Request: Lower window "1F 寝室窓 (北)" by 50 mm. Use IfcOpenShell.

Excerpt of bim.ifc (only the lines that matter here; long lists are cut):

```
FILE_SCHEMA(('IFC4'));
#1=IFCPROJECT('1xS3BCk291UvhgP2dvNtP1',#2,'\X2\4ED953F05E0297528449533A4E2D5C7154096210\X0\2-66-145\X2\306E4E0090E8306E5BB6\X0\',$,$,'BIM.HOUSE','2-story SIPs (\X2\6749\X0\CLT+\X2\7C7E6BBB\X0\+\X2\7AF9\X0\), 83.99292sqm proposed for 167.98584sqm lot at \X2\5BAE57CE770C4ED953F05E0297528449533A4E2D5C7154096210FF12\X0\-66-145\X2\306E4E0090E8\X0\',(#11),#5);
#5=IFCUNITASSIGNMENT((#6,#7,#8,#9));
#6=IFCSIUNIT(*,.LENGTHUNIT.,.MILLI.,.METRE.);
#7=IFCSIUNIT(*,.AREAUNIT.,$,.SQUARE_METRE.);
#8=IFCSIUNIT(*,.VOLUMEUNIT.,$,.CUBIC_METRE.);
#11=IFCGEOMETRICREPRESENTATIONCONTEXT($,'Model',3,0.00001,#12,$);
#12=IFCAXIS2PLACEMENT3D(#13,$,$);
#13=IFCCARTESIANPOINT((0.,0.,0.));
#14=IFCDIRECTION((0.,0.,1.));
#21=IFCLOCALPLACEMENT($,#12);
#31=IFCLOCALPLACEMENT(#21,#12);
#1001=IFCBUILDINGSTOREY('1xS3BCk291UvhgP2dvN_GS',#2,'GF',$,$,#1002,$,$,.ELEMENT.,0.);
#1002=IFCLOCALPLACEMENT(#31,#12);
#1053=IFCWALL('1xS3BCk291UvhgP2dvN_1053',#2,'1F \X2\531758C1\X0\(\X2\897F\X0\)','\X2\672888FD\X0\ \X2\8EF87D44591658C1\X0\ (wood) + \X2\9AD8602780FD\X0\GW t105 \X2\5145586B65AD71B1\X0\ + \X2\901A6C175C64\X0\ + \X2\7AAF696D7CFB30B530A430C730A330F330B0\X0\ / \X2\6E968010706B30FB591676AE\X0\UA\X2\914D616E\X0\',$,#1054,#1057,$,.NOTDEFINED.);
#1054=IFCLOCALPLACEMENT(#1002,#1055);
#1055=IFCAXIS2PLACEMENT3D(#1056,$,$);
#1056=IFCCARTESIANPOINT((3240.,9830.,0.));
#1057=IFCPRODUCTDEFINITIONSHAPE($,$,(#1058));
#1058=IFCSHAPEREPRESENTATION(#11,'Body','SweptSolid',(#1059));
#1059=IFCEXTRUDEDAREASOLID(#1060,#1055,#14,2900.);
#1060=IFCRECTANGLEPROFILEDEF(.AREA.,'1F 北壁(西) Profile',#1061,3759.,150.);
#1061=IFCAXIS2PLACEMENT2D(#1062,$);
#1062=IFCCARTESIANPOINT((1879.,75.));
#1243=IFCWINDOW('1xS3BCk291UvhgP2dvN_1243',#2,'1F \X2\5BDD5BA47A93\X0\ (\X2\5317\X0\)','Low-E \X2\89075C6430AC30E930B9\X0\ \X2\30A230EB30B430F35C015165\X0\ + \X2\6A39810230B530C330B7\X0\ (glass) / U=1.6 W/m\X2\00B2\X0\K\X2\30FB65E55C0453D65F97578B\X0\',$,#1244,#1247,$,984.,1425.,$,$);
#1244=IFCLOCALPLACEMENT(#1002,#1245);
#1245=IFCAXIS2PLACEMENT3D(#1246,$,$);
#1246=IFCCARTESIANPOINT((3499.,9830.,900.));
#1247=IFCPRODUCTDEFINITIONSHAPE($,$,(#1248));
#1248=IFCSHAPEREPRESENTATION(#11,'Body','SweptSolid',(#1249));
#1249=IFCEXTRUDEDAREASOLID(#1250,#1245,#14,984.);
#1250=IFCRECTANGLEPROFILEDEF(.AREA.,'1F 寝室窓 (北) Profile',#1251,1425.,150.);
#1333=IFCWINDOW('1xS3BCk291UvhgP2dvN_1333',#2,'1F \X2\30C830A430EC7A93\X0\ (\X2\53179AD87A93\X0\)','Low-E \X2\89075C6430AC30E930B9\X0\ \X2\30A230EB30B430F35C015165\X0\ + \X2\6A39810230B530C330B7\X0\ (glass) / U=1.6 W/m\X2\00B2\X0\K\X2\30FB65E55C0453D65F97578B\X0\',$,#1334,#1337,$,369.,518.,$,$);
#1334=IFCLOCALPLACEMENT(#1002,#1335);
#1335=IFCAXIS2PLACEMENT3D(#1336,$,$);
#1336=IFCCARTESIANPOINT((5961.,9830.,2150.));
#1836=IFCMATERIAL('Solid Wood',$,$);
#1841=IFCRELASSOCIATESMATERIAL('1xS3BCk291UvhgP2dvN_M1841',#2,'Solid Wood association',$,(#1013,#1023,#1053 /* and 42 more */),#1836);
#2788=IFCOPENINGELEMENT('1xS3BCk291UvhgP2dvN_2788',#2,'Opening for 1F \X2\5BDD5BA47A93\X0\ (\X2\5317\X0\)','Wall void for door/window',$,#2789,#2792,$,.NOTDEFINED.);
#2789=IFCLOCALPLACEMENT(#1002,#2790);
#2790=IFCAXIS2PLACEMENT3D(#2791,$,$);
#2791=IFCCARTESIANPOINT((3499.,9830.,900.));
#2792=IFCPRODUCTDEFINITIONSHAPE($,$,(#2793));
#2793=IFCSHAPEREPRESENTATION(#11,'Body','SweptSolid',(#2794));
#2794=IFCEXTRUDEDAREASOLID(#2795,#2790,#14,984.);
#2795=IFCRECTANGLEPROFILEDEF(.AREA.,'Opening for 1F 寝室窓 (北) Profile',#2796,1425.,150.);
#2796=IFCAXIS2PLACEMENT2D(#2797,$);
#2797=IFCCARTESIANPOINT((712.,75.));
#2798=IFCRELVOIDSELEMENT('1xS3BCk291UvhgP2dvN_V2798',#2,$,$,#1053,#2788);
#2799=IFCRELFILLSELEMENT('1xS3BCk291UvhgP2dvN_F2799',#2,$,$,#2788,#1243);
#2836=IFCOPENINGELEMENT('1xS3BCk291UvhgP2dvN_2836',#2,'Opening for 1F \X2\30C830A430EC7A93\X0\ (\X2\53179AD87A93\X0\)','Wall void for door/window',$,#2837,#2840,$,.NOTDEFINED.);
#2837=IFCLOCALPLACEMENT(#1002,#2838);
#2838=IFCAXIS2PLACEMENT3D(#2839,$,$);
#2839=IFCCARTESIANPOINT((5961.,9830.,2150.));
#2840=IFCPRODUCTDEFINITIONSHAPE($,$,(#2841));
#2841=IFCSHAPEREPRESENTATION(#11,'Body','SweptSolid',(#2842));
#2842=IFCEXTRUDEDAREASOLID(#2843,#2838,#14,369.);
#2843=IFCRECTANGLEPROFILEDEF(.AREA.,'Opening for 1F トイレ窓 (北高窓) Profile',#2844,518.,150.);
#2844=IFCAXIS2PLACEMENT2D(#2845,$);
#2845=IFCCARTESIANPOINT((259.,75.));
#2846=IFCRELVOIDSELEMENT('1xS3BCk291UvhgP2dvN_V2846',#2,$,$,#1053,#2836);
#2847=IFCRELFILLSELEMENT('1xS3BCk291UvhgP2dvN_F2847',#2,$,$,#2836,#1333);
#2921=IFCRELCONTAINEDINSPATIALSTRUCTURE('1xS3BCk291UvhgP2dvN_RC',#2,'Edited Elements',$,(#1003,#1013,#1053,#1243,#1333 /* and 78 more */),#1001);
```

```python
import numpy as np
import ifcopenshell
import ifcopenshell.api.geometry
import ifcopenshell.util.placement
import ifcopenshell.util.unit

model = ifcopenshell.open("bim.ifc")
unit_scale = ifcopenshell.util.unit.calculate_unit_scale(model)

window = model.by_guid("1xS3BCk291UvhgP2dvN_1243")
opening = window.FillsVoids[0].RelatingOpeningElement
dz = -50.0

shift = np.array([0.0, 0.0, dz])
# The window is not placed relative to its opening, so move both.
for product in (opening, window):
    matrix = ifcopenshell.util.placement.get_local_placement(product.ObjectPlacement)
    matrix[:3, 3] += shift
    ifcopenshell.api.geometry.edit_object_placement(model, product=product, matrix=matrix, is_si=False)

print(f"moved by {dz * unit_scale:+.3f} m")

model.write("bim_edited.ifc")
```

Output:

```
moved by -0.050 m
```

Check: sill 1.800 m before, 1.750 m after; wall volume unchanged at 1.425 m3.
